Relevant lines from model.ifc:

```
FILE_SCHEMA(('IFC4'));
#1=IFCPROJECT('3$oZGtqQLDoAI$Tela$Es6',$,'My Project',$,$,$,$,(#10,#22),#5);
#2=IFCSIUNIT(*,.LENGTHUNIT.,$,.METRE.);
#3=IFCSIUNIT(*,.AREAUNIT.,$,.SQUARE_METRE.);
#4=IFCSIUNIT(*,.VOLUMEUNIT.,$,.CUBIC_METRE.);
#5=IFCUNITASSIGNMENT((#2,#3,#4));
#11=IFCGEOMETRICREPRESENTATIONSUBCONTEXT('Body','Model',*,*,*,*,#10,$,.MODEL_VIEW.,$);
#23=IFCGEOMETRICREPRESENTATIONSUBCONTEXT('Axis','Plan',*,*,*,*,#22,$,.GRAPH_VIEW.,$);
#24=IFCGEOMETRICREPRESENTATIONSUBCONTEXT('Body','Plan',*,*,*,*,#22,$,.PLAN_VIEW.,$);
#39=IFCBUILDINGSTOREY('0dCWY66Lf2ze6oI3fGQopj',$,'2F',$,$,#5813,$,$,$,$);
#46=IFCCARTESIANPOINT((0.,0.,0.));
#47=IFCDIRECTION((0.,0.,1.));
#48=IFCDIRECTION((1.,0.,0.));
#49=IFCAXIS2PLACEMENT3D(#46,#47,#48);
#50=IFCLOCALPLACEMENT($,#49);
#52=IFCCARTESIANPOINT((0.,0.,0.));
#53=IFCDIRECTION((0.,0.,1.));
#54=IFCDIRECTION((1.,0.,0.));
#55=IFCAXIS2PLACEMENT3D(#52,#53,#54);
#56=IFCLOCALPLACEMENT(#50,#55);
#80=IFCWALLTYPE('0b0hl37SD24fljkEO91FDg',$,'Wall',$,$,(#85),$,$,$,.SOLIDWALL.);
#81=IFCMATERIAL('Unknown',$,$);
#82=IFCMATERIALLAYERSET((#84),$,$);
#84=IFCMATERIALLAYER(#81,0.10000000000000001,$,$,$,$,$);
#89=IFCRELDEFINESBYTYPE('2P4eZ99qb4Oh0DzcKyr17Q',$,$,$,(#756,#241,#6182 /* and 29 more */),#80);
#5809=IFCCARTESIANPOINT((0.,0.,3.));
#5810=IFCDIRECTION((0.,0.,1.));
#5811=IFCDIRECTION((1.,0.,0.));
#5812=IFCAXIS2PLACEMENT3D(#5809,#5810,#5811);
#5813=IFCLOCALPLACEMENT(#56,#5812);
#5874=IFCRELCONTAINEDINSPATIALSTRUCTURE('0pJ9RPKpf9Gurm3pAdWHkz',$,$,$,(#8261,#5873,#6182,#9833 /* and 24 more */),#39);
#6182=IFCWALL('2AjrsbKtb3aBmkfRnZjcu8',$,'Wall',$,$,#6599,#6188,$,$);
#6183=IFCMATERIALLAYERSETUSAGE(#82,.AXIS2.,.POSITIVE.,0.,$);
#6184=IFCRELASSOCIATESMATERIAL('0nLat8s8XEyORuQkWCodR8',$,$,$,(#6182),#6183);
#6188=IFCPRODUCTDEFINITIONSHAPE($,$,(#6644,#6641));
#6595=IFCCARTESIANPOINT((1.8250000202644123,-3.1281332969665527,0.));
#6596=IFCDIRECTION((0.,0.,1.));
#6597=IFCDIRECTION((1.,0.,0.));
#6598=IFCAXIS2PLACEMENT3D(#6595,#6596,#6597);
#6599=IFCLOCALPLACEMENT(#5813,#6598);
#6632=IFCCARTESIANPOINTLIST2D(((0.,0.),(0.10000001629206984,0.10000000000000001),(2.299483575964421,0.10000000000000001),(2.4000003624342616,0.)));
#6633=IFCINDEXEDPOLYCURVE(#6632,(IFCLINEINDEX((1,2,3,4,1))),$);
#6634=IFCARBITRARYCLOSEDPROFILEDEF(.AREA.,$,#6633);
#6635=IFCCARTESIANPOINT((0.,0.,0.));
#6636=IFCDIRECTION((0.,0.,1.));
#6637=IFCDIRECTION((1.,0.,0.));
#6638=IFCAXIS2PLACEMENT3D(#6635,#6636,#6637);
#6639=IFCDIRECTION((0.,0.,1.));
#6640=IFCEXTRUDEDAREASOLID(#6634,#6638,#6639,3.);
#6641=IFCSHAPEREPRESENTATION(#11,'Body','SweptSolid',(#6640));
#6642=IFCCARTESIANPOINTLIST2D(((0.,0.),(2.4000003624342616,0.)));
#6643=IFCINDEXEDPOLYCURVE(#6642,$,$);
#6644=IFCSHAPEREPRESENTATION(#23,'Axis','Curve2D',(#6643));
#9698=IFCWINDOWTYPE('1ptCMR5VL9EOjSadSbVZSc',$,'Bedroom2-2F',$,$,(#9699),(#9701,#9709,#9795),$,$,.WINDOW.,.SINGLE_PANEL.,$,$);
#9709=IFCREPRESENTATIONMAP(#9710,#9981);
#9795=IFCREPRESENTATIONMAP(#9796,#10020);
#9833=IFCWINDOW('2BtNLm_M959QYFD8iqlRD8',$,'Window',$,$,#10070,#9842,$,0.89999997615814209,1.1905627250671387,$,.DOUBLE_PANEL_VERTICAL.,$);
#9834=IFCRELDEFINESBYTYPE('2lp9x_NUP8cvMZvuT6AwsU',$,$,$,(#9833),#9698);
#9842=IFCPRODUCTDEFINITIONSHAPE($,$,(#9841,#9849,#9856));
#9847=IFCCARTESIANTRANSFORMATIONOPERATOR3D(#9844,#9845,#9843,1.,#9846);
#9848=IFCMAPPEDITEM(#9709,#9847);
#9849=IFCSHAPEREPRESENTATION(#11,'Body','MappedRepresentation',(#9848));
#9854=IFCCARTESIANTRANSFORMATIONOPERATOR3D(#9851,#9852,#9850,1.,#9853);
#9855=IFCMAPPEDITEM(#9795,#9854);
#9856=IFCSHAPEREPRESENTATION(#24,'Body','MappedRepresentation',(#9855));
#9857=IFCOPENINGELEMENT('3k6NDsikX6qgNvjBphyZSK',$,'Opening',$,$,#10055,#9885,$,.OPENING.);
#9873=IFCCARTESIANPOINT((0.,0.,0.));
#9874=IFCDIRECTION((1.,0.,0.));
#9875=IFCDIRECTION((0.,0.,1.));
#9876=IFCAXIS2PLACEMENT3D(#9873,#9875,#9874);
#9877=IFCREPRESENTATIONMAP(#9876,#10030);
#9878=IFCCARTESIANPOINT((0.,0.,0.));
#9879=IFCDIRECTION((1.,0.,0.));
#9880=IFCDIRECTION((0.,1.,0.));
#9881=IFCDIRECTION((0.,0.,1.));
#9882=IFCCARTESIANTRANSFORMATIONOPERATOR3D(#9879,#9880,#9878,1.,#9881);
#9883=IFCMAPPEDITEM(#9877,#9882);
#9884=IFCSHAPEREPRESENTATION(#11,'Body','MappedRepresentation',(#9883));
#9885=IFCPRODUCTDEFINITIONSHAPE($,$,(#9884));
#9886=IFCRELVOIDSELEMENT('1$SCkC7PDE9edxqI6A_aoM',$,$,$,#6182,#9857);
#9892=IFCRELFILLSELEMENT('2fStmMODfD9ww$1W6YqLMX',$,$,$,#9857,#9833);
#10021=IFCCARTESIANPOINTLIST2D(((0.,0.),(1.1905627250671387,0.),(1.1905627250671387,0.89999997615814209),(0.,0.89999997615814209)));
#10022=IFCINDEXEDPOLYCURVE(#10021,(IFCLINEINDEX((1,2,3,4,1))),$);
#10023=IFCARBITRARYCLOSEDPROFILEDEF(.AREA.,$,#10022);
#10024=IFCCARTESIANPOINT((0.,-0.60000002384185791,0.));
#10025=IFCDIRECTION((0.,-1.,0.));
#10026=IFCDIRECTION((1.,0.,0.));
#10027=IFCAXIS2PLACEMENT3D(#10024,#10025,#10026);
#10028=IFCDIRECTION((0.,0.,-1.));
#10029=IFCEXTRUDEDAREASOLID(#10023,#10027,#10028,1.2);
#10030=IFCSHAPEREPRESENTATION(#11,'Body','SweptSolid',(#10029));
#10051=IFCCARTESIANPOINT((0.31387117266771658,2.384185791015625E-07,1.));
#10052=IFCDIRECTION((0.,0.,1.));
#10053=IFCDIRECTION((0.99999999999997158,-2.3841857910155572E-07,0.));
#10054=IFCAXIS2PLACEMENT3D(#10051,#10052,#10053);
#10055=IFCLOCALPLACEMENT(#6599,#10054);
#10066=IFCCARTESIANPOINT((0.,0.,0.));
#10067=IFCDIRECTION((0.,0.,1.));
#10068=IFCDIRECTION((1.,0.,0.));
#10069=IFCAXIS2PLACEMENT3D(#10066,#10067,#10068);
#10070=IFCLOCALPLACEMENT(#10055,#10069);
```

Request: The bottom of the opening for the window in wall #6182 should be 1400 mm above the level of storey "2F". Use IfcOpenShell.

```python
import numpy as np
import ifcopenshell
import ifcopenshell.api.geometry
import ifcopenshell.geom
import ifcopenshell.util.element
import ifcopenshell.util.placement
import ifcopenshell.util.shape
import ifcopenshell.util.unit

model = ifcopenshell.open("model.ifc")
unit_scale = ifcopenshell.util.unit.calculate_unit_scale(model)

window = model.by_id(9833)
opening = window.FillsVoids[0].RelatingOpeningElement
storey = ifcopenshell.util.element.get_container(window, ifc_class="IfcBuildingStorey")
level = ifcopenshell.util.placement.get_local_placement(storey.ObjectPlacement)[2, 3]

# The opening's origin need not be at the sill, so measure its lowest point.
shape = ifcopenshell.geom.create_shape(ifcopenshell.geom.settings(), opening)
bottom = ifcopenshell.util.shape.get_shape_bottom_elevation(shape, shape.geometry) / unit_scale
dz = level + 1.4 / unit_scale - bottom

shift = np.array([0.0, 0.0, dz])
# The window is placed relative to its opening, so it follows when the opening moves.
matrix = ifcopenshell.util.placement.get_local_placement(opening.ObjectPlacement)
matrix[:3, 3] += shift
ifcopenshell.api.geometry.edit_object_placement(
    model, product=opening, matrix=matrix, is_si=False, should_transform_children=True
)

print(f"moved by {dz * unit_scale:+.3f} m")

model.write("model_v2.ifc")
```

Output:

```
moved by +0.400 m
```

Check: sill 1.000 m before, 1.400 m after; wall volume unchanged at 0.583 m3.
